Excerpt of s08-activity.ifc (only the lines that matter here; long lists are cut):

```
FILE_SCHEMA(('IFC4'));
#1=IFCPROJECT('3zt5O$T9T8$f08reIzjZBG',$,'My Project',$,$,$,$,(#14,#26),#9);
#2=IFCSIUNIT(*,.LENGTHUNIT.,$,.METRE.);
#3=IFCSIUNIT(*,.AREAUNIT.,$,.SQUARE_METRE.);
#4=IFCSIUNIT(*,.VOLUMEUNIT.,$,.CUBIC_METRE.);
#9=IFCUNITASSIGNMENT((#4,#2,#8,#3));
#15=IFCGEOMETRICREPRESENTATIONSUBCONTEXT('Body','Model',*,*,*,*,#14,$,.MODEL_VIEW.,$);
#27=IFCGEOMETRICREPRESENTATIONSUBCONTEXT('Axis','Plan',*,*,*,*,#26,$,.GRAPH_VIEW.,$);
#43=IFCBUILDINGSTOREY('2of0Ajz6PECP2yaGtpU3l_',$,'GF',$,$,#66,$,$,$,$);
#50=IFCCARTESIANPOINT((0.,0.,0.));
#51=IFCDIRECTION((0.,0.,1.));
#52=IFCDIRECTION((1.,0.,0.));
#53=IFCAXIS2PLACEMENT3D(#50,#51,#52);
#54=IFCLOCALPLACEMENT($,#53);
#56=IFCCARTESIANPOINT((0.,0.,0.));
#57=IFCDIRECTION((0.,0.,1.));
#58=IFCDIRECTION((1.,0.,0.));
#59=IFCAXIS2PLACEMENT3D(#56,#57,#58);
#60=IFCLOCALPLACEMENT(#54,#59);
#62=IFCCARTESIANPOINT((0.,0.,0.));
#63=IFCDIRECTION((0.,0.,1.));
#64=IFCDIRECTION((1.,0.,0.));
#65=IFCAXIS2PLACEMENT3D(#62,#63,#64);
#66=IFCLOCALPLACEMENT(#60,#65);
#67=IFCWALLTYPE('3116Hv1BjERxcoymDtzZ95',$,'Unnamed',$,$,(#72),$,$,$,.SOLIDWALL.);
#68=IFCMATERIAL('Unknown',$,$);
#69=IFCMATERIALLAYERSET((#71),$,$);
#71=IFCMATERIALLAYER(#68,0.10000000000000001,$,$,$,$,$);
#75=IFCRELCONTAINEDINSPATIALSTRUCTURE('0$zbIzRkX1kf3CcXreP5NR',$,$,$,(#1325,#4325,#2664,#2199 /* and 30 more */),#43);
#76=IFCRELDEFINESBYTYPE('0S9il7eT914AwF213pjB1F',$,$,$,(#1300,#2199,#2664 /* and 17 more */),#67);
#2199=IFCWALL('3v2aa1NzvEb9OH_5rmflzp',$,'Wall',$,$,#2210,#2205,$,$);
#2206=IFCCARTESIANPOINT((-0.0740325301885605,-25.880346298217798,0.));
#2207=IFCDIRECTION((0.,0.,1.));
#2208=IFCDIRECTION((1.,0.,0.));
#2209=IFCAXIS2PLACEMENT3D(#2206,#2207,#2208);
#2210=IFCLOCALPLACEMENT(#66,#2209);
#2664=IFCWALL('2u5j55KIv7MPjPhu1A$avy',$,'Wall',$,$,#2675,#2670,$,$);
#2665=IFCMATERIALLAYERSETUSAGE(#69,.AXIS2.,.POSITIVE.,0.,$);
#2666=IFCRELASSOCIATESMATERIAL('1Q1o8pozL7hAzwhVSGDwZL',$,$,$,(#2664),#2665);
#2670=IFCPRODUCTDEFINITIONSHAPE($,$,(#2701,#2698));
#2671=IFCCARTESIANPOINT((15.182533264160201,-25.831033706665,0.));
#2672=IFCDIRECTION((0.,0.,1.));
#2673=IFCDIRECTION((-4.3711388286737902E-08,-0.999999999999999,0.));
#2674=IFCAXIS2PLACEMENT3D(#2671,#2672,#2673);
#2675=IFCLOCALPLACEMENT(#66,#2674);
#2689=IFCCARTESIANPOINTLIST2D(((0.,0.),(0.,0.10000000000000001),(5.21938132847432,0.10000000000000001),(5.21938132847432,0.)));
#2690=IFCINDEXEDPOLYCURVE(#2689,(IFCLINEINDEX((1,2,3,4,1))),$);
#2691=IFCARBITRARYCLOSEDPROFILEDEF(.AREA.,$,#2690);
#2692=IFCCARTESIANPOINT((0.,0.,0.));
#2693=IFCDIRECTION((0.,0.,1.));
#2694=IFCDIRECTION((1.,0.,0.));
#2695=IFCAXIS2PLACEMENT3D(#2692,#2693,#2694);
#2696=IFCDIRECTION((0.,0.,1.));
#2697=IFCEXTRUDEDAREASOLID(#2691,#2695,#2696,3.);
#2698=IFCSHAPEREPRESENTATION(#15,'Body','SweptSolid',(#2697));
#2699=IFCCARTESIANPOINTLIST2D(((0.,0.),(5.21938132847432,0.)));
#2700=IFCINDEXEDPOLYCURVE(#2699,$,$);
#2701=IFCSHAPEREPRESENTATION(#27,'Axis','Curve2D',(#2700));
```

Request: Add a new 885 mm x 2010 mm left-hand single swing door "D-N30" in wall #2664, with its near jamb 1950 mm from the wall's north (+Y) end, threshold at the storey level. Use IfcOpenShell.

```python
import numpy as np
import ifcopenshell
import ifcopenshell.api.feature
import ifcopenshell.api.geometry
import ifcopenshell.api.root
import ifcopenshell.api.spatial
import ifcopenshell.geom
import ifcopenshell.util.element
import ifcopenshell.util.placement
import ifcopenshell.util.representation
import ifcopenshell.util.shape
import ifcopenshell.util.unit

model = ifcopenshell.open("s08-activity.ifc")
unit_scale = ifcopenshell.util.unit.calculate_unit_scale(model)
settings = ifcopenshell.geom.settings()


def volume(element):
    """Net volume in cubic metres, openings subtracted."""
    shape = ifcopenshell.geom.create_shape(settings, element)
    return ifcopenshell.util.shape.get_volume(shape.geometry)


wall = model.by_guid("2u5j55KIv7MPjPhu1A$avy")
storey = ifcopenshell.util.element.get_container(wall, ifc_class="IfcBuildingStorey")
context = ifcopenshell.util.representation.get_context(model, "Model", "Body", "MODEL_VIEW")
before = volume(wall)

width, height, from_end, sill = 0.885, 2.01, 1.95, 0.0  # metres

# The wall runs along its own X axis, and the end named is its -X end.
wall_shape = ifcopenshell.geom.create_shape(settings, wall)
x, y, z = ifcopenshell.util.shape.get_vertices(wall_shape.geometry).T
start = x.min() + from_end
face, thickness = float(y.min()), float(y.max() - y.min())
wall_matrix = ifcopenshell.util.placement.get_local_placement(wall.ObjectPlacement)
level = ifcopenshell.util.placement.get_local_placement(storey.ObjectPlacement)[2, 3]


def in_wall(x, y):
    """Placement at x, y metres in the wall's axes, at sill height."""
    matrix = wall_matrix.copy()
    matrix[:, 3] = wall_matrix @ np.array([x / unit_scale, y / unit_scale, 0.0, 1.0])
    matrix[2, 3] = level + sill / unit_scale
    return matrix


# Opening: a box that overshoots both wall faces by 50 mm.
opening = ifcopenshell.api.root.create_entity(model, ifc_class="IfcOpeningElement", predefined_type="OPENING")
box = ifcopenshell.api.geometry.add_wall_representation(
    model, context=context, length=width, height=height, thickness=thickness + 0.1
)
ifcopenshell.api.geometry.assign_representation(model, product=opening, representation=box)
ifcopenshell.api.geometry.edit_object_placement(model, product=opening, matrix=in_wall(start, face - 0.05), is_si=False)
ifcopenshell.api.feature.add_feature(model, feature=opening, element=wall)

door = ifcopenshell.api.root.create_entity(model, ifc_class="IfcDoor", name="D-N30", predefined_type="DOOR")
door.OverallWidth, door.OverallHeight = width / unit_scale, height / unit_scale
door.OperationType = "SINGLE_SWING_LEFT"
body = ifcopenshell.api.geometry.add_door_representation(
    model,
    context=context,
    overall_width=door.OverallWidth,
    overall_height=door.OverallHeight,
    operation_type="SINGLE_SWING_LEFT",
    lining_properties={"LiningDepth": thickness / unit_scale, "ThresholdDepth": thickness / unit_scale},
)
ifcopenshell.api.geometry.assign_representation(model, product=door, representation=body)
ifcopenshell.api.spatial.assign_container(model, products=[door], relating_structure=storey)
ifcopenshell.api.feature.add_filling(model, opening=opening, element=door)

# The lining spans the wall, so the door starts at the wall face.
ifcopenshell.api.geometry.edit_object_placement(model, product=door, matrix=in_wall(start, face), is_si=False)

after = volume(wall)

print(f"wall volume {before:.3f} -> {after:.3f} m3")

model.write("s08-activity_edited.ifc")
```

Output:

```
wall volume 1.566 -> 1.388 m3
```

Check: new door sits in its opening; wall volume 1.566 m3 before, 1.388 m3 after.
